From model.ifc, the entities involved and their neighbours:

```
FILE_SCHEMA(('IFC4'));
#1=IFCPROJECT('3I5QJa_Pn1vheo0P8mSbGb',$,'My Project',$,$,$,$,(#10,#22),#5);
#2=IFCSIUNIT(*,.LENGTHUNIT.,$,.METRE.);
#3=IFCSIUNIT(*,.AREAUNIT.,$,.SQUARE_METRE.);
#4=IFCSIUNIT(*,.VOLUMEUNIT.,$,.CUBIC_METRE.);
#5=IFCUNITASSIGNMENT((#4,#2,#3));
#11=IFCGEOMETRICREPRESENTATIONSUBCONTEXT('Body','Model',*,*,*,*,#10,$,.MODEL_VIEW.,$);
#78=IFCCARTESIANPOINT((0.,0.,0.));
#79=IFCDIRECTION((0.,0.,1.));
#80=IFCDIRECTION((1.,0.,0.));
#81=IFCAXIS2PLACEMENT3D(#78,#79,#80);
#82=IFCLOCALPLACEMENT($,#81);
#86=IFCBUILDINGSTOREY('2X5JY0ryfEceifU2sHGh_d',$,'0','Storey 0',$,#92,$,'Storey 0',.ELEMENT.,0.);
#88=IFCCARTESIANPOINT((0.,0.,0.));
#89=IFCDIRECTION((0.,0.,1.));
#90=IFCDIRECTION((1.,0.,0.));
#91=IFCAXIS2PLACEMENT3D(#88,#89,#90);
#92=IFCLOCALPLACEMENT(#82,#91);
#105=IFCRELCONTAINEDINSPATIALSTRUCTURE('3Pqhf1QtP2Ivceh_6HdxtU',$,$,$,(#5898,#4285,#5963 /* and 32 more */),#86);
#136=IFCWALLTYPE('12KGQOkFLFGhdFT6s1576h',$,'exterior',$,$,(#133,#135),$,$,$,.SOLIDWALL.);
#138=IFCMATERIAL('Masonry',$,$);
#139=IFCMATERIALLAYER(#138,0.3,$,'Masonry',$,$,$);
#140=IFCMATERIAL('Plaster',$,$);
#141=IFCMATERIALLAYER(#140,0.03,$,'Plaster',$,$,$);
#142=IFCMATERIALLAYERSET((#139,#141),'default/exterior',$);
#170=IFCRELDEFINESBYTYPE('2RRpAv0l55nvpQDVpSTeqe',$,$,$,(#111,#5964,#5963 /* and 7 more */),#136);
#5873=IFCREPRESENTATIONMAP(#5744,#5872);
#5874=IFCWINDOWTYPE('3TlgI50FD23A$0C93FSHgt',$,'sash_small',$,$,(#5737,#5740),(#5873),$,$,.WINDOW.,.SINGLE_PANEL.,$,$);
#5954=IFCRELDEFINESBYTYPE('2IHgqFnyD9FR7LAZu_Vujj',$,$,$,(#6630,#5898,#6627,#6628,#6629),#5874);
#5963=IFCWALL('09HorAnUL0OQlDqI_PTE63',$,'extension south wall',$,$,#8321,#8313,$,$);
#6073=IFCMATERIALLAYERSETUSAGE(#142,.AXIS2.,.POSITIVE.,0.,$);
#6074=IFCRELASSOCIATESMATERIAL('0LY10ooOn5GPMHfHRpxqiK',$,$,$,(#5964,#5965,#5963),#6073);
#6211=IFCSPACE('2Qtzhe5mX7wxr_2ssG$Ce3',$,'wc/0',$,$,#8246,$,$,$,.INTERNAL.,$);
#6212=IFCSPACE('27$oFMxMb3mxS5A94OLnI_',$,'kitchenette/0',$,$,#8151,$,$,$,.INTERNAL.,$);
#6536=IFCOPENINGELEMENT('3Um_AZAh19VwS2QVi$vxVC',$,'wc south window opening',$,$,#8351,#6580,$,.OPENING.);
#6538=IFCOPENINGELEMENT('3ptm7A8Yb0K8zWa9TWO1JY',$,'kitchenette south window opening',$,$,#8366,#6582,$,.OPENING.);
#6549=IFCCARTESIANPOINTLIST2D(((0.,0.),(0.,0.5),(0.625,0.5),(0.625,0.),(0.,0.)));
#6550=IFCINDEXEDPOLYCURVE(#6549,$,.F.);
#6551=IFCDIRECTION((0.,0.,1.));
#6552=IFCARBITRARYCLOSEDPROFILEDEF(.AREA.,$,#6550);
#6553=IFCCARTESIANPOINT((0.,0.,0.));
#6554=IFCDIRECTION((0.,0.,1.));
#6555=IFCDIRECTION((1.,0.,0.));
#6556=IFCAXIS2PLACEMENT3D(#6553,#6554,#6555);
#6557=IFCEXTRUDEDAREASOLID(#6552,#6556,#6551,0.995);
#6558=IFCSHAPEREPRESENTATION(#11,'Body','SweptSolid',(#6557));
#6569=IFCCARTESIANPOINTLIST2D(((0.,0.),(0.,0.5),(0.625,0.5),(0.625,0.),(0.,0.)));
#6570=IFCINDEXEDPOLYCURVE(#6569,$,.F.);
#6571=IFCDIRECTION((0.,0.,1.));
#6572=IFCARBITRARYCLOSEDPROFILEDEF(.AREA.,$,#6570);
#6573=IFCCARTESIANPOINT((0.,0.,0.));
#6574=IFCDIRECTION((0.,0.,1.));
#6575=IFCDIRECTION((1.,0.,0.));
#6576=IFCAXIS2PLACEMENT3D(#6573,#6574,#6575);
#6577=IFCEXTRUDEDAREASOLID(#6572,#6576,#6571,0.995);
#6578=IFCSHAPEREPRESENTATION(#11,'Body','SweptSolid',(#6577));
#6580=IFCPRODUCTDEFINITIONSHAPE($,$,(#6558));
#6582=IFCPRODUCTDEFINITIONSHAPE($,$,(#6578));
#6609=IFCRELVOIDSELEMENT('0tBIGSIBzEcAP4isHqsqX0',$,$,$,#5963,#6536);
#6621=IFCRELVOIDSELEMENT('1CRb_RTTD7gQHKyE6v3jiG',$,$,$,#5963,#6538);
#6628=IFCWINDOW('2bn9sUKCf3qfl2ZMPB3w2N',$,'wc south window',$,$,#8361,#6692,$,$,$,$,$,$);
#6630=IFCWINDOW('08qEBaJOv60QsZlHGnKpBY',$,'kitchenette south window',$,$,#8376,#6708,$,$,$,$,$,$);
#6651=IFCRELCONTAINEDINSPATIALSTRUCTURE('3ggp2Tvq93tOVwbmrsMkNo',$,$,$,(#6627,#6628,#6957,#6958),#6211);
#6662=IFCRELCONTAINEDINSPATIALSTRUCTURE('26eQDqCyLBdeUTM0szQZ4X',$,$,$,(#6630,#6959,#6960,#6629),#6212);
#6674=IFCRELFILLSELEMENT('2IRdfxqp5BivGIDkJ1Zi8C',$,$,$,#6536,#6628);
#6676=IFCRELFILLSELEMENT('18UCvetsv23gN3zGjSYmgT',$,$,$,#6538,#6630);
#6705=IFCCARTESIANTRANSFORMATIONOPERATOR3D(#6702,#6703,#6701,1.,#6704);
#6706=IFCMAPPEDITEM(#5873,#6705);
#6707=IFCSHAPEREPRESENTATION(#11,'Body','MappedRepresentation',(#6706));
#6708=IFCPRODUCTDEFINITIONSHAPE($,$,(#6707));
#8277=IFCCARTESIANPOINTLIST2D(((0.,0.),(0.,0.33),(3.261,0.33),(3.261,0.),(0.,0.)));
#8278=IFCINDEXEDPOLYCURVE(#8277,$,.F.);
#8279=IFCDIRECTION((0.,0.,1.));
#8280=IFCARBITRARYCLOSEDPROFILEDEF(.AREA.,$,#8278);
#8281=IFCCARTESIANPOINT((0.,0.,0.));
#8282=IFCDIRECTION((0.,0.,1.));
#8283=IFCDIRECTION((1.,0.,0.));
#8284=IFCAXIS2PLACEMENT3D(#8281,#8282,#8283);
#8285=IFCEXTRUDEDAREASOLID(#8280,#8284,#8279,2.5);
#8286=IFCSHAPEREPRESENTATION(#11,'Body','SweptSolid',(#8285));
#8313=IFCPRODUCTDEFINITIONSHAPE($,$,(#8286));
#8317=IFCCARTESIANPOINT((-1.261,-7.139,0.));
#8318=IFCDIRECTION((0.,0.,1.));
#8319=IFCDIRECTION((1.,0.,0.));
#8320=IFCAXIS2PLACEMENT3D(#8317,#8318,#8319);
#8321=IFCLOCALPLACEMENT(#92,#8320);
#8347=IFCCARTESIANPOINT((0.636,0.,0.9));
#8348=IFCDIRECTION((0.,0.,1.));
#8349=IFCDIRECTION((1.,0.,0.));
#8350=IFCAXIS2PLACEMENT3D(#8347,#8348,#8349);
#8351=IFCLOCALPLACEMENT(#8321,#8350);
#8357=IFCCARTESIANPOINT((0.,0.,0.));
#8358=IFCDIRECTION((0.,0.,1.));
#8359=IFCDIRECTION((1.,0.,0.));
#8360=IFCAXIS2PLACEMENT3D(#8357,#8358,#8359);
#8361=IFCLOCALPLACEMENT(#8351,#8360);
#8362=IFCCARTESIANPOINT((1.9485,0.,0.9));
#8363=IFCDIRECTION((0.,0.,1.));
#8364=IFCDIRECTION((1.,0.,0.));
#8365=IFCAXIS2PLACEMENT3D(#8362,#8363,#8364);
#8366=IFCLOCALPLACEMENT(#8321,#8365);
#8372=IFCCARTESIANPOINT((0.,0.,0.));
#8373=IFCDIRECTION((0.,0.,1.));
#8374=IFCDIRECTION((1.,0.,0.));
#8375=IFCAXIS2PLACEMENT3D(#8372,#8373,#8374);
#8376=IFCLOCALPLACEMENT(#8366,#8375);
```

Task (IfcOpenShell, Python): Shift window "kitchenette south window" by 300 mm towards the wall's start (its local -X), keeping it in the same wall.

```python
import ifcopenshell
import ifcopenshell.api.geometry
import ifcopenshell.util.placement
import ifcopenshell.util.unit

model = ifcopenshell.open("model.ifc")
unit_scale = ifcopenshell.util.unit.calculate_unit_scale(model)

window = model.by_guid("08qEBaJOv60QsZlHGnKpBY")
opening = window.FillsVoids[0].RelatingOpeningElement
wall = opening.VoidsElements[0].RelatingBuildingElement

wall_matrix = ifcopenshell.util.placement.get_local_placement(wall.ObjectPlacement)
shift = wall_matrix[:3, 0] * -0.3 / unit_scale
before = ifcopenshell.util.placement.get_local_placement(window.ObjectPlacement)[:3, 3].copy()

# The window is placed relative to its opening, so it follows when the opening moves.
matrix = ifcopenshell.util.placement.get_local_placement(opening.ObjectPlacement)
matrix[:3, 3] += shift
ifcopenshell.api.geometry.edit_object_placement(
    model, product=opening, matrix=matrix, is_si=False, should_transform_children=True
)

after = ifcopenshell.util.placement.get_local_placement(window.ObjectPlacement)[:3, 3]
print("window moved by", (after - before).round(3) + 0.0)

model.write("model_rev.ifc")
```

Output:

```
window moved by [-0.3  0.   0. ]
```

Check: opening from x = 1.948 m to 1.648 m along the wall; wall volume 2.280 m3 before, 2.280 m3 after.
